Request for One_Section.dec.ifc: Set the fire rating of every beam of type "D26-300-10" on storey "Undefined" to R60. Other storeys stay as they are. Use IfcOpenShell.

First a look at what the model holds.

```python
import ifcopenshell
import ifcopenshell.util.element

model = ifcopenshell.open("One_Section.dec.ifc")
print(model.schema)
storey = next(s for s in model.by_type("IfcBuildingStorey") if s.Name == "Undefined")
beams = [e for e in ifcopenshell.util.element.get_decomposition(storey) if e.is_a("IfcBeam")]
seen = {}
for e in beams:
    element_type = ifcopenshell.util.element.get_type(e)
    key = (element_type.Name if element_type != e and element_type else None, ifcopenshell.util.element.get_pset(e, "Pset_BeamCommon", "FireRating"))
    seen[key] = seen.get(key, 0) + 1
for (name, value), count in sorted(seen.items(), key=str):
    print(count, "x", name, "|", value)
```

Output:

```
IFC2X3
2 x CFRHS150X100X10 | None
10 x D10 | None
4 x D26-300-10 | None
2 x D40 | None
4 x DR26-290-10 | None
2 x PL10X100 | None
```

```python
import ifcopenshell
import ifcopenshell.api.pset
import ifcopenshell.util.element

model = ifcopenshell.open("One_Section.dec.ifc")

storey = next(s for s in model.by_type("IfcBuildingStorey") if s.Name == "Undefined")
beams = [e for e in ifcopenshell.util.element.get_decomposition(storey) if e.is_a("IfcBeam")]

count = 0
for e in beams:
    element_type = ifcopenshell.util.element.get_type(e)
    if element_type in (None, e) or element_type.Name != "D26-300-10":
        continue
    found = ifcopenshell.util.element.get_pset(e, "Pset_BeamCommon", should_inherit=False)
    if found:
        pset = model.by_id(found["id"])
        if len(ifcopenshell.util.element.get_elements_by_pset(pset)) > 1:
            pset = ifcopenshell.api.pset.unshare_pset(model, products=[e], pset=pset)[0]
    else:
        pset = ifcopenshell.api.pset.add_pset(model, product=e, name="Pset_BeamCommon")
    ifcopenshell.api.pset.edit_pset(model, pset=pset, properties={"FireRating": "R60"})
    count += 1

print(count, "beams updated")

model.write("One_Section.dec_v2.ifc")
```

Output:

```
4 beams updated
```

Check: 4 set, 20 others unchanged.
